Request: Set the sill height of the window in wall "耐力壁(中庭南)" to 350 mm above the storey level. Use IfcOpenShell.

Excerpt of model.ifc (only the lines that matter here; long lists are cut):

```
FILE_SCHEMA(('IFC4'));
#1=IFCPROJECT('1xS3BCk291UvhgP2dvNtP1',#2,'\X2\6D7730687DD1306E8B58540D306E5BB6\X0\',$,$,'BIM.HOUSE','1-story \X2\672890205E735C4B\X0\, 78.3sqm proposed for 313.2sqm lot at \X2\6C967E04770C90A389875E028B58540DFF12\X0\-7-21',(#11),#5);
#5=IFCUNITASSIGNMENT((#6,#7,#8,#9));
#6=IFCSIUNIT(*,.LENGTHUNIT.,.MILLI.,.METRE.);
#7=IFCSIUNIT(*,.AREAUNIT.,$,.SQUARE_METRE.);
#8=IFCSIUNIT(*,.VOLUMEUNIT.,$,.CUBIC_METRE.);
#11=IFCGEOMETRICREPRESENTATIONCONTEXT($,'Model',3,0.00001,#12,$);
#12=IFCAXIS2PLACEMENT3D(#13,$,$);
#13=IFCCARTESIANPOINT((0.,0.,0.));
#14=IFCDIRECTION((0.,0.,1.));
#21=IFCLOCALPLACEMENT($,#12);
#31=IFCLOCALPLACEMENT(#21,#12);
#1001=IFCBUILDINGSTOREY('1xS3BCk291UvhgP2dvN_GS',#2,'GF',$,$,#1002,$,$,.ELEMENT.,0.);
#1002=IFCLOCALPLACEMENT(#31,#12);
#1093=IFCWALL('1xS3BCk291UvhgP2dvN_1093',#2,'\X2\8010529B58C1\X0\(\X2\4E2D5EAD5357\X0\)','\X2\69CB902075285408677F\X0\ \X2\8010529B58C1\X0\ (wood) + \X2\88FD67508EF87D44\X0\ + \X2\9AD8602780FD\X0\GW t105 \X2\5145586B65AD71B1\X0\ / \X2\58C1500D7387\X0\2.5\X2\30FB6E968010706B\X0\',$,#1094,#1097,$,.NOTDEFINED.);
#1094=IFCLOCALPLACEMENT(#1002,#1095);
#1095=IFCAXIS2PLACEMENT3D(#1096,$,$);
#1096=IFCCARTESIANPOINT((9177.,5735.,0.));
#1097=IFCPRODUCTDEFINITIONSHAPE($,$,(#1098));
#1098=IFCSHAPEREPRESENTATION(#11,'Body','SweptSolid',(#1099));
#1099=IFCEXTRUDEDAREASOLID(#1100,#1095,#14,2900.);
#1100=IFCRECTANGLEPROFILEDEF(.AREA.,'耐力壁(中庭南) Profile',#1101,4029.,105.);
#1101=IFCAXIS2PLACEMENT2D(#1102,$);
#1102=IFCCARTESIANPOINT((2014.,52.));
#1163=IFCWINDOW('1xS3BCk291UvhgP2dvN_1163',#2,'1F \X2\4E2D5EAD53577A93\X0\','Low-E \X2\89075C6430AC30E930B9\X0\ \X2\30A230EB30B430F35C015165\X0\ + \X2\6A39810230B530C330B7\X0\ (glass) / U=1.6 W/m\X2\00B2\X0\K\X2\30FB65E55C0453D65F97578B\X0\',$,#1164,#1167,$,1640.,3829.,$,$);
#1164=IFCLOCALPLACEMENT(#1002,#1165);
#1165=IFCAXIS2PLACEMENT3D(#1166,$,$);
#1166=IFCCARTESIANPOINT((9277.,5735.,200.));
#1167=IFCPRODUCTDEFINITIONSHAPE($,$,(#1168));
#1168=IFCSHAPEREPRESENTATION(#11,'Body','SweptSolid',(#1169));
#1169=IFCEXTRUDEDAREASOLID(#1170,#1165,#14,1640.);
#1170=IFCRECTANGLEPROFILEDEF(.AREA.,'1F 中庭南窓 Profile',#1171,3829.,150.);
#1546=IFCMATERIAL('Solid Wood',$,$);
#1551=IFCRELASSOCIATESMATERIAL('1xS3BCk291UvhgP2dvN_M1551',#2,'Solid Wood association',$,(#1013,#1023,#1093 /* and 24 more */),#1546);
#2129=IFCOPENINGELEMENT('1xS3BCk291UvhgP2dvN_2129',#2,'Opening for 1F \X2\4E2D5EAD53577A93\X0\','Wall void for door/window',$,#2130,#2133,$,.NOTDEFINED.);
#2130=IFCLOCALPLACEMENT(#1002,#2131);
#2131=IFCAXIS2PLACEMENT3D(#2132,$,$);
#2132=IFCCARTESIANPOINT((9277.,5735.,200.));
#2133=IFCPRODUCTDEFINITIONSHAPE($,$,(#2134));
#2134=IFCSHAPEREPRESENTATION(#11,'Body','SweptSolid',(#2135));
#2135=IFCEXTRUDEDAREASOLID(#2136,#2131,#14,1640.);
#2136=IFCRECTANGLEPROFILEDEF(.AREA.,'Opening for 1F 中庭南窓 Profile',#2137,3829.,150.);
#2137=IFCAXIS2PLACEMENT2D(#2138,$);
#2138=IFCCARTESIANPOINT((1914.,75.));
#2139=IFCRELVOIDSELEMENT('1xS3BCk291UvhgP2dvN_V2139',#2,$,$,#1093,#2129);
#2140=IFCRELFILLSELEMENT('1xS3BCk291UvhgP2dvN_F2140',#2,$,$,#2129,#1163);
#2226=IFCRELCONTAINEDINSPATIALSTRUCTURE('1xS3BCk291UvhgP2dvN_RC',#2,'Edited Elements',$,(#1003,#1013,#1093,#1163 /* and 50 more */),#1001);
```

```python
import numpy as np
import ifcopenshell
import ifcopenshell.api.geometry
import ifcopenshell.geom
import ifcopenshell.util.element
import ifcopenshell.util.placement
import ifcopenshell.util.shape
import ifcopenshell.util.unit

model = ifcopenshell.open("model.ifc")
unit_scale = ifcopenshell.util.unit.calculate_unit_scale(model)

window = model.by_guid("1xS3BCk291UvhgP2dvN_1163")
opening = window.FillsVoids[0].RelatingOpeningElement
storey = ifcopenshell.util.element.get_container(window, ifc_class="IfcBuildingStorey")
level = ifcopenshell.util.placement.get_local_placement(storey.ObjectPlacement)[2, 3]

# The opening's origin need not be at the sill, so measure its lowest point.
shape = ifcopenshell.geom.create_shape(ifcopenshell.geom.settings(), opening)
bottom = ifcopenshell.util.shape.get_shape_bottom_elevation(shape, shape.geometry) / unit_scale
dz = level + 0.35 / unit_scale - bottom

shift = np.array([0.0, 0.0, dz])
# The window is not placed relative to its opening, so move both.
for product in (opening, window):
    matrix = ifcopenshell.util.placement.get_local_placement(product.ObjectPlacement)
    matrix[:3, 3] += shift
    ifcopenshell.api.geometry.edit_object_placement(model, product=product, matrix=matrix, is_si=False)

print(f"moved by {dz * unit_scale:+.3f} m")

model.write("model_updated.ifc")
```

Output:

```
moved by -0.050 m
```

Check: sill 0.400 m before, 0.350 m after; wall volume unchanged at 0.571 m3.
